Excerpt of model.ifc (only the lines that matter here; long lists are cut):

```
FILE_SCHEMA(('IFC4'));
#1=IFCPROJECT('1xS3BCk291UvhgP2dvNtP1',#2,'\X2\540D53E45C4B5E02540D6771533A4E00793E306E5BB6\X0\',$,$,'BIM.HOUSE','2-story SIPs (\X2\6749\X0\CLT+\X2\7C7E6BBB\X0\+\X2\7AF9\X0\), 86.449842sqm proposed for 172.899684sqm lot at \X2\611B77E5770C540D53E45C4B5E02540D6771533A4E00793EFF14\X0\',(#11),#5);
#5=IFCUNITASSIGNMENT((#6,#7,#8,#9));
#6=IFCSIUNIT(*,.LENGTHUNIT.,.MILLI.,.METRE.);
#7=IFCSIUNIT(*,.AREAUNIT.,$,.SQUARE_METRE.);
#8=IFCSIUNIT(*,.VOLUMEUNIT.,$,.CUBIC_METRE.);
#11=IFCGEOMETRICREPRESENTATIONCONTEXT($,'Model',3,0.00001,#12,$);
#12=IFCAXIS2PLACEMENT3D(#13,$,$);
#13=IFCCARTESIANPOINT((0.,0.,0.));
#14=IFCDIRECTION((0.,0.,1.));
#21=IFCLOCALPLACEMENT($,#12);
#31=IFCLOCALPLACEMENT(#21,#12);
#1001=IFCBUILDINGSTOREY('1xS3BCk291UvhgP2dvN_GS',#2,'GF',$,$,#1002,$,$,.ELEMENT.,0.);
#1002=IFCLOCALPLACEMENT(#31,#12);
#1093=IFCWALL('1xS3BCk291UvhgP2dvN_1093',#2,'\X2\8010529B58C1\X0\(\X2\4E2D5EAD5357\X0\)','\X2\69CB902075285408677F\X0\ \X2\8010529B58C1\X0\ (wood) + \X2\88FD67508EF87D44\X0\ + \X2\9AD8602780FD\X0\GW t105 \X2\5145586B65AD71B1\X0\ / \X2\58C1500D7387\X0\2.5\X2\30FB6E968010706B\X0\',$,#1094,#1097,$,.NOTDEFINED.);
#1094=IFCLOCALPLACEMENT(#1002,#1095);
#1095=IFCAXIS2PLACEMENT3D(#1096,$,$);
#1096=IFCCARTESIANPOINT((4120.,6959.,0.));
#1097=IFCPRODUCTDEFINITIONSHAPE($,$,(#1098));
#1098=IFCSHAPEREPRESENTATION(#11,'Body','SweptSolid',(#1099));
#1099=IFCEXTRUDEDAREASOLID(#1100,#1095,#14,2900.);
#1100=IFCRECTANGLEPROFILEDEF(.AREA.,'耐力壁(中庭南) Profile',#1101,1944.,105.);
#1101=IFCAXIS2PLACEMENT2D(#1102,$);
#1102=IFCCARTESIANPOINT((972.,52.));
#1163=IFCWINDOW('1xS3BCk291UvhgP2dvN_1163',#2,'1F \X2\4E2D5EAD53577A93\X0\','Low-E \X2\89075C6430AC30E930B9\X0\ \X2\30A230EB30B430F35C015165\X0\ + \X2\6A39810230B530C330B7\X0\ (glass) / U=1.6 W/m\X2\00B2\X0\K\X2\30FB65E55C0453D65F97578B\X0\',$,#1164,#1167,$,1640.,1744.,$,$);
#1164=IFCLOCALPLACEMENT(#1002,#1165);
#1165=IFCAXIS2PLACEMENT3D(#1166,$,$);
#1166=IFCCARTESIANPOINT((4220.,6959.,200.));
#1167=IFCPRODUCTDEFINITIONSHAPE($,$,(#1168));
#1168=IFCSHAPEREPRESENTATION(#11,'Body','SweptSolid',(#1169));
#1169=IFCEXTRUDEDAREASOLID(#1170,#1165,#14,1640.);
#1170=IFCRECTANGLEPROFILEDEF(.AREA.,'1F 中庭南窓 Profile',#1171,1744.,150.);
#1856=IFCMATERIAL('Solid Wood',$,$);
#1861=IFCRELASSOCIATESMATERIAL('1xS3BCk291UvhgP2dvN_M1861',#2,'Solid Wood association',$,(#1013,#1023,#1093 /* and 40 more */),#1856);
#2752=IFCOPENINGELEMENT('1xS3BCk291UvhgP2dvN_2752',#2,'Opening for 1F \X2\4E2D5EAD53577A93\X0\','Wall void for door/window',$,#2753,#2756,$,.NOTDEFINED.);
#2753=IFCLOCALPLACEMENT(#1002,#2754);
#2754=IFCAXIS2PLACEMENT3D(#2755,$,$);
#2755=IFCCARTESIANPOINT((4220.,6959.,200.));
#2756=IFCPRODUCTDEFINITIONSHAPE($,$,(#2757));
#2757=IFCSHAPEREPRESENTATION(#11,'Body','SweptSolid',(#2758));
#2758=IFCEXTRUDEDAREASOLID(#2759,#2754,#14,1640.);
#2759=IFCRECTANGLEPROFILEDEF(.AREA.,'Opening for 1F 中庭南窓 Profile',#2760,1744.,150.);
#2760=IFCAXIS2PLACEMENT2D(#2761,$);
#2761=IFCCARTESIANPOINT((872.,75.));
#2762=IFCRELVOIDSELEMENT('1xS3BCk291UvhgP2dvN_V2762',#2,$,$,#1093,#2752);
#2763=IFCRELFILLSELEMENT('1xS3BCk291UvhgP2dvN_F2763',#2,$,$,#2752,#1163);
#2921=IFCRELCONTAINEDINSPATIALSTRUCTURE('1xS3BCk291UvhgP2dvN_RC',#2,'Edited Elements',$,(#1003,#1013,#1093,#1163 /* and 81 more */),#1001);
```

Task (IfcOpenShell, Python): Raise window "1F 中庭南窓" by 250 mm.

```python
import numpy as np
import ifcopenshell
import ifcopenshell.api.geometry
import ifcopenshell.util.placement
import ifcopenshell.util.unit

model = ifcopenshell.open("model.ifc")
unit_scale = ifcopenshell.util.unit.calculate_unit_scale(model)

window = model.by_id(1163)
opening = window.FillsVoids[0].RelatingOpeningElement
dz = 250.0

shift = np.array([0.0, 0.0, dz])
# The window is not placed relative to its opening, so move both.
for product in (opening, window):
    matrix = ifcopenshell.util.placement.get_local_placement(product.ObjectPlacement)
    matrix[:3, 3] += shift
    ifcopenshell.api.geometry.edit_object_placement(model, product=product, matrix=matrix, is_si=False)

print(f"moved by {dz * unit_scale:+.3f} m")

model.write("model-out.ifc")
```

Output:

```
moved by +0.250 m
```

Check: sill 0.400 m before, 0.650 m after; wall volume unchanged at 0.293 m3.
